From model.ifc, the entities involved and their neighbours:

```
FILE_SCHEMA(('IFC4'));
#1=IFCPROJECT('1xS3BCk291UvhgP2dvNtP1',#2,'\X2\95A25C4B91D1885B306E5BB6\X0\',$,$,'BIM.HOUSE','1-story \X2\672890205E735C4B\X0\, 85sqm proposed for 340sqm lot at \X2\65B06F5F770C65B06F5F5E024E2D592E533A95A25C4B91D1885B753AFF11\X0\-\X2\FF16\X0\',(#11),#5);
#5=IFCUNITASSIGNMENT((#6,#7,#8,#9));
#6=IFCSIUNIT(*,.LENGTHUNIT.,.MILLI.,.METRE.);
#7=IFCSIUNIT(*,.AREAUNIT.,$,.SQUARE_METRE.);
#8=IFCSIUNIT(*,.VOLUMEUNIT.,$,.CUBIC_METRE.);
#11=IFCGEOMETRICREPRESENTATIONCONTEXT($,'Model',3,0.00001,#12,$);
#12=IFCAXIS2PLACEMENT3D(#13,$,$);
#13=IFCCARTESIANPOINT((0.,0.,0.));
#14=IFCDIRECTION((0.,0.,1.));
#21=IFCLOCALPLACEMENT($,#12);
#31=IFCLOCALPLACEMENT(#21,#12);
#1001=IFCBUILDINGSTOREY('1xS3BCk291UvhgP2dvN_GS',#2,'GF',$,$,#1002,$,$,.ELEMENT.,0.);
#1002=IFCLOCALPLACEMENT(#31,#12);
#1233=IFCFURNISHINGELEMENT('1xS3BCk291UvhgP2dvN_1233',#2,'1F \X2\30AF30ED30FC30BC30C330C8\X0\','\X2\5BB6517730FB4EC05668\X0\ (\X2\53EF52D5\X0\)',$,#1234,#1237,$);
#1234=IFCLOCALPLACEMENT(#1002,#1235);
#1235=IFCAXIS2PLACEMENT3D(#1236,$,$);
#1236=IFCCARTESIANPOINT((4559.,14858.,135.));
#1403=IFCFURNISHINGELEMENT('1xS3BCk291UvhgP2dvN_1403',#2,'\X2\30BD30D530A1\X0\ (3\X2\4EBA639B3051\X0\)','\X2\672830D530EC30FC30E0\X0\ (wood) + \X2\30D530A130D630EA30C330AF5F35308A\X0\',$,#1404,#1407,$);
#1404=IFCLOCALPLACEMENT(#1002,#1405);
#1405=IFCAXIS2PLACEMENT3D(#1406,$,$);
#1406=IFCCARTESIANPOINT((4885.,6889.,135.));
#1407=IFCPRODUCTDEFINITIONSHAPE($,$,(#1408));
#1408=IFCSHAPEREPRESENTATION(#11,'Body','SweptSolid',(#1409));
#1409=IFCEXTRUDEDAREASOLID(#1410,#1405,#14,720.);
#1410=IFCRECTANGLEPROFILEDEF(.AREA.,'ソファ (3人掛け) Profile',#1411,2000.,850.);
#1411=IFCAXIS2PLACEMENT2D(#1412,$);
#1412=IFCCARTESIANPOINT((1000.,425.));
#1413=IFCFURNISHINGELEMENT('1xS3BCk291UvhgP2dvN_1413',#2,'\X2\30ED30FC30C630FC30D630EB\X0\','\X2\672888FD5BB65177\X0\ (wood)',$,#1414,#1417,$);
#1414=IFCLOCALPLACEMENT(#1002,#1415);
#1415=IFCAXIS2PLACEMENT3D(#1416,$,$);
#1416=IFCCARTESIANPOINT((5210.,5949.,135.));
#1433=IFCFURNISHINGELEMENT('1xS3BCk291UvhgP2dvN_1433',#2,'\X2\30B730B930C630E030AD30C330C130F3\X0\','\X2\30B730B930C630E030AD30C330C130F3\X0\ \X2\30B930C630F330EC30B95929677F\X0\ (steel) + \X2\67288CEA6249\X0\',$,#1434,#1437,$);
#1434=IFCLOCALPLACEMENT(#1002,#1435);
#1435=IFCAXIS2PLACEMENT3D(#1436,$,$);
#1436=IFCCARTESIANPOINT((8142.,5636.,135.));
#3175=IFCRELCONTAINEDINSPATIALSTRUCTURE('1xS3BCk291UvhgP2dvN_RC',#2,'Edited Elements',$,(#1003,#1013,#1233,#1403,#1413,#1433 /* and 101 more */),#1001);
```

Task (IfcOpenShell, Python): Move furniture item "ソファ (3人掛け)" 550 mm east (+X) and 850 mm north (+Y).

```python
import ifcopenshell
import ifcopenshell.api.geometry
import ifcopenshell.util.placement

model = ifcopenshell.open("model.ifc")

item = model.by_id(1403)
matrix = ifcopenshell.util.placement.get_local_placement(item.ObjectPlacement)
matrix[0, 3] += 550.0
matrix[1, 3] += 850.0
ifcopenshell.api.geometry.edit_object_placement(model, product=item, matrix=matrix, is_si=False)

print(ifcopenshell.util.placement.get_local_placement(item.ObjectPlacement).round(3) + 0.0)

model.write("model-out.ifc")
```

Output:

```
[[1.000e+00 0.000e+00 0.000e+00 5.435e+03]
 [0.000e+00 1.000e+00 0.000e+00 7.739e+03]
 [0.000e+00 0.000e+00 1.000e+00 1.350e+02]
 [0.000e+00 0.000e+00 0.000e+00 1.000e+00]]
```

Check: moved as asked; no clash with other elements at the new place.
